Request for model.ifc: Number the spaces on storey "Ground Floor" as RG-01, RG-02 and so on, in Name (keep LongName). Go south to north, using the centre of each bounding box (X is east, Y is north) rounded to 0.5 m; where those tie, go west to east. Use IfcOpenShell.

First a look at what the model holds.

```python
import ifcopenshell
import ifcopenshell.util.element
import ifcopenshell.util.placement

model = ifcopenshell.open("model.ifc")
print(model.schema)
storey = next(s for s in model.by_type("IfcBuildingStorey") if s.Name == "Ground Floor")
spaces = [e for e in ifcopenshell.util.element.get_decomposition(storey) if e.is_a("IfcSpace")]
for e in sorted(spaces, key=lambda e: e.id()):
    origin = ifcopenshell.util.placement.get_local_placement(e.ObjectPlacement)[:3, 3]
    print(e.id(), e.Name, e.LongName, origin.round(2) + 0.0, sep=" | ")
```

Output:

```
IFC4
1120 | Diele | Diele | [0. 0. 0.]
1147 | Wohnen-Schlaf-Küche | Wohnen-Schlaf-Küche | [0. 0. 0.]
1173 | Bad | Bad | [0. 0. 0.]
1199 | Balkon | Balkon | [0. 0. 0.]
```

```python
import ifcopenshell
import ifcopenshell.geom
import ifcopenshell.util.element
import ifcopenshell.util.shape

model = ifcopenshell.open("model.ifc")
settings = ifcopenshell.geom.settings()
settings.set("use-world-coords", True)


def centre(element):
    shape = ifcopenshell.geom.create_shape(settings, element)
    return ifcopenshell.util.shape.get_bbox_centroid(shape.geometry)


storey = next(s for s in model.by_type("IfcBuildingStorey") if s.Name == "Ground Floor")
spaces = [e for e in ifcopenshell.util.element.get_decomposition(storey) if e.is_a("IfcSpace")]

# Insertion points can sit at a corner or the storey origin, so sort by the geometry (in metres).
centres = {e: centre(e) for e in spaces}
spaces.sort(key=lambda e: (round(centres[e][1] / 0.5), centres[e][0]))

for i, e in enumerate(spaces, start=1):
    number = f"RG-{i:02d}"
    e.Name = number
    print(e.id(), number)

model.write("model_edited.ifc")
```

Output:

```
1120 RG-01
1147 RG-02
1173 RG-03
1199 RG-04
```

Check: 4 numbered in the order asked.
